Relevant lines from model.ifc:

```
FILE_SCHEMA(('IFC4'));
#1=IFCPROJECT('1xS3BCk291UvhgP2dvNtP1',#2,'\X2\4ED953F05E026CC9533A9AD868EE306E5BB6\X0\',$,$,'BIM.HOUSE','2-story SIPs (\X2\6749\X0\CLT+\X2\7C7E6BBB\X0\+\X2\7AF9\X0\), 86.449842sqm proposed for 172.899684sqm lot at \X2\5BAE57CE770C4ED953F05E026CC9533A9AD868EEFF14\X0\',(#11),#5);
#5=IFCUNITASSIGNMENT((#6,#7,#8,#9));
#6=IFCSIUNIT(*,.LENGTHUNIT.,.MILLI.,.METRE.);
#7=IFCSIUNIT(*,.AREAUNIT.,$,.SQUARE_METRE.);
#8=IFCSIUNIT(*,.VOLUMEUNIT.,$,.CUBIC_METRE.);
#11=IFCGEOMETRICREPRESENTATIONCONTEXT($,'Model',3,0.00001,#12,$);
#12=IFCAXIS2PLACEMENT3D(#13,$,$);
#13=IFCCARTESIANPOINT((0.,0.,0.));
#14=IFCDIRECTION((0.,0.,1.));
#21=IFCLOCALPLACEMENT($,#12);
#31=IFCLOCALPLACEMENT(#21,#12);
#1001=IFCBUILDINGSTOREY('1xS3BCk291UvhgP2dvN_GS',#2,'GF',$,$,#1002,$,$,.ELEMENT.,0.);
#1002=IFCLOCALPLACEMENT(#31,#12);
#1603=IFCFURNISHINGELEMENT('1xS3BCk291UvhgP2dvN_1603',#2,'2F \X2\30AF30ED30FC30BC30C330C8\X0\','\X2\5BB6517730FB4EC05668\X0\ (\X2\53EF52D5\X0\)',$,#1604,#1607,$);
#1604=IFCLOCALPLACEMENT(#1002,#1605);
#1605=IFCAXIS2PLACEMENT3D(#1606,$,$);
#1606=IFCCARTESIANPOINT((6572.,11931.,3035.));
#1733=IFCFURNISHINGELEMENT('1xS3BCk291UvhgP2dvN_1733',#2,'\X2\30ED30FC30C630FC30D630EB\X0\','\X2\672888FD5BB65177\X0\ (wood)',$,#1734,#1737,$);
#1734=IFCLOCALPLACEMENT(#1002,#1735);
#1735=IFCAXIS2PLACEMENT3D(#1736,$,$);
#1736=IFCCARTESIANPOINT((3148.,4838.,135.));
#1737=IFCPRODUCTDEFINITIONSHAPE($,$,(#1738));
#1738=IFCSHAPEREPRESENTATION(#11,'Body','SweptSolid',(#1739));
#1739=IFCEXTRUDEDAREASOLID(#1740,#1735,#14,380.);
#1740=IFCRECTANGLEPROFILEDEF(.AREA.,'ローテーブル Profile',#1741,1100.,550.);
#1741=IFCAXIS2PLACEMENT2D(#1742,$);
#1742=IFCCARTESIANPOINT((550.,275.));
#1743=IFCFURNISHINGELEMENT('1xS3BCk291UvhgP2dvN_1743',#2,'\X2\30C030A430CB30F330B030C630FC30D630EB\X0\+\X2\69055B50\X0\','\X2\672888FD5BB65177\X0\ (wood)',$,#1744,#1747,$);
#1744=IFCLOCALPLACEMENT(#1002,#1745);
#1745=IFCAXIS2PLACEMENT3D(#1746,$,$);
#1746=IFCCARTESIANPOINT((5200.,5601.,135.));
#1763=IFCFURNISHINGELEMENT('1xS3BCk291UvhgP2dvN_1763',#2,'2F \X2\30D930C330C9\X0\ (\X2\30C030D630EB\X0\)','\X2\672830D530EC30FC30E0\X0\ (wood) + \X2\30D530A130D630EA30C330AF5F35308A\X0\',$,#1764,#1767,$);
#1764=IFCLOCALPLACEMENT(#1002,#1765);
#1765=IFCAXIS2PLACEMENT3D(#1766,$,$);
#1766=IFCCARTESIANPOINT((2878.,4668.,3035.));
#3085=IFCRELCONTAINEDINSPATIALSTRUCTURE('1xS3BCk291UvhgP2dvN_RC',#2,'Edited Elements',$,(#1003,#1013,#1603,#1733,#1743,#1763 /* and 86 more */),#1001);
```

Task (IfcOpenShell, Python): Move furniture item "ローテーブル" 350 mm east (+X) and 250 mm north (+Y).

```python
import ifcopenshell
import ifcopenshell.api.geometry
import ifcopenshell.util.placement
import ifcopenshell.util.unit

model = ifcopenshell.open("model.ifc")
unit_scale = ifcopenshell.util.unit.calculate_unit_scale(model)

item = model.by_guid("1xS3BCk291UvhgP2dvN_1733")
matrix = ifcopenshell.util.placement.get_local_placement(item.ObjectPlacement)
matrix[0, 3] += 0.35 / unit_scale
matrix[1, 3] += 0.25 / unit_scale
ifcopenshell.api.geometry.edit_object_placement(model, product=item, matrix=matrix, is_si=False)

print(ifcopenshell.util.placement.get_local_placement(item.ObjectPlacement).round(3) + 0.0)

model.write("model-out.ifc")
```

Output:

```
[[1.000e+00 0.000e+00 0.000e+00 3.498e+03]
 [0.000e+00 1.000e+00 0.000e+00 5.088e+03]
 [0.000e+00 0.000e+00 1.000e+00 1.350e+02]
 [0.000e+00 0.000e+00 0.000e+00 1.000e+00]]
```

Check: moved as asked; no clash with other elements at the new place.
